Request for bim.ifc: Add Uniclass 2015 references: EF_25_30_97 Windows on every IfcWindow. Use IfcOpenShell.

First a look at what the model holds.

```python
import ifcopenshell

model = ifcopenshell.open("bim.ifc")
print(model.schema)
print("classifications:", [c.Name for c in model.by_type("IfcClassification")])
for ifc_class in ("IfcDoor", "IfcRoof", "IfcStair", "IfcWall", "IfcWindow"):
    print(ifc_class, len(model.by_type(ifc_class)))
```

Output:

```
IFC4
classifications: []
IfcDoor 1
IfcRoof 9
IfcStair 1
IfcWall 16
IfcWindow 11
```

```python
import ifcopenshell
import ifcopenshell.api.classification

model = ifcopenshell.open("bim.ifc")

system = ifcopenshell.api.classification.add_classification(model, classification="Uniclass 2015")

codes = {
    "IfcWindow": ("EF_25_30_97", "Windows"),
}
for ifc_class, (code, name) in codes.items():
    products = model.by_type(ifc_class)
    ifcopenshell.api.classification.add_reference(
        model, products=products, classification=system, identification=code, name=name
    )
    print(code, len(products))

model.write("bim-out.ifc")
```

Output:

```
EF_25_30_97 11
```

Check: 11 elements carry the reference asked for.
